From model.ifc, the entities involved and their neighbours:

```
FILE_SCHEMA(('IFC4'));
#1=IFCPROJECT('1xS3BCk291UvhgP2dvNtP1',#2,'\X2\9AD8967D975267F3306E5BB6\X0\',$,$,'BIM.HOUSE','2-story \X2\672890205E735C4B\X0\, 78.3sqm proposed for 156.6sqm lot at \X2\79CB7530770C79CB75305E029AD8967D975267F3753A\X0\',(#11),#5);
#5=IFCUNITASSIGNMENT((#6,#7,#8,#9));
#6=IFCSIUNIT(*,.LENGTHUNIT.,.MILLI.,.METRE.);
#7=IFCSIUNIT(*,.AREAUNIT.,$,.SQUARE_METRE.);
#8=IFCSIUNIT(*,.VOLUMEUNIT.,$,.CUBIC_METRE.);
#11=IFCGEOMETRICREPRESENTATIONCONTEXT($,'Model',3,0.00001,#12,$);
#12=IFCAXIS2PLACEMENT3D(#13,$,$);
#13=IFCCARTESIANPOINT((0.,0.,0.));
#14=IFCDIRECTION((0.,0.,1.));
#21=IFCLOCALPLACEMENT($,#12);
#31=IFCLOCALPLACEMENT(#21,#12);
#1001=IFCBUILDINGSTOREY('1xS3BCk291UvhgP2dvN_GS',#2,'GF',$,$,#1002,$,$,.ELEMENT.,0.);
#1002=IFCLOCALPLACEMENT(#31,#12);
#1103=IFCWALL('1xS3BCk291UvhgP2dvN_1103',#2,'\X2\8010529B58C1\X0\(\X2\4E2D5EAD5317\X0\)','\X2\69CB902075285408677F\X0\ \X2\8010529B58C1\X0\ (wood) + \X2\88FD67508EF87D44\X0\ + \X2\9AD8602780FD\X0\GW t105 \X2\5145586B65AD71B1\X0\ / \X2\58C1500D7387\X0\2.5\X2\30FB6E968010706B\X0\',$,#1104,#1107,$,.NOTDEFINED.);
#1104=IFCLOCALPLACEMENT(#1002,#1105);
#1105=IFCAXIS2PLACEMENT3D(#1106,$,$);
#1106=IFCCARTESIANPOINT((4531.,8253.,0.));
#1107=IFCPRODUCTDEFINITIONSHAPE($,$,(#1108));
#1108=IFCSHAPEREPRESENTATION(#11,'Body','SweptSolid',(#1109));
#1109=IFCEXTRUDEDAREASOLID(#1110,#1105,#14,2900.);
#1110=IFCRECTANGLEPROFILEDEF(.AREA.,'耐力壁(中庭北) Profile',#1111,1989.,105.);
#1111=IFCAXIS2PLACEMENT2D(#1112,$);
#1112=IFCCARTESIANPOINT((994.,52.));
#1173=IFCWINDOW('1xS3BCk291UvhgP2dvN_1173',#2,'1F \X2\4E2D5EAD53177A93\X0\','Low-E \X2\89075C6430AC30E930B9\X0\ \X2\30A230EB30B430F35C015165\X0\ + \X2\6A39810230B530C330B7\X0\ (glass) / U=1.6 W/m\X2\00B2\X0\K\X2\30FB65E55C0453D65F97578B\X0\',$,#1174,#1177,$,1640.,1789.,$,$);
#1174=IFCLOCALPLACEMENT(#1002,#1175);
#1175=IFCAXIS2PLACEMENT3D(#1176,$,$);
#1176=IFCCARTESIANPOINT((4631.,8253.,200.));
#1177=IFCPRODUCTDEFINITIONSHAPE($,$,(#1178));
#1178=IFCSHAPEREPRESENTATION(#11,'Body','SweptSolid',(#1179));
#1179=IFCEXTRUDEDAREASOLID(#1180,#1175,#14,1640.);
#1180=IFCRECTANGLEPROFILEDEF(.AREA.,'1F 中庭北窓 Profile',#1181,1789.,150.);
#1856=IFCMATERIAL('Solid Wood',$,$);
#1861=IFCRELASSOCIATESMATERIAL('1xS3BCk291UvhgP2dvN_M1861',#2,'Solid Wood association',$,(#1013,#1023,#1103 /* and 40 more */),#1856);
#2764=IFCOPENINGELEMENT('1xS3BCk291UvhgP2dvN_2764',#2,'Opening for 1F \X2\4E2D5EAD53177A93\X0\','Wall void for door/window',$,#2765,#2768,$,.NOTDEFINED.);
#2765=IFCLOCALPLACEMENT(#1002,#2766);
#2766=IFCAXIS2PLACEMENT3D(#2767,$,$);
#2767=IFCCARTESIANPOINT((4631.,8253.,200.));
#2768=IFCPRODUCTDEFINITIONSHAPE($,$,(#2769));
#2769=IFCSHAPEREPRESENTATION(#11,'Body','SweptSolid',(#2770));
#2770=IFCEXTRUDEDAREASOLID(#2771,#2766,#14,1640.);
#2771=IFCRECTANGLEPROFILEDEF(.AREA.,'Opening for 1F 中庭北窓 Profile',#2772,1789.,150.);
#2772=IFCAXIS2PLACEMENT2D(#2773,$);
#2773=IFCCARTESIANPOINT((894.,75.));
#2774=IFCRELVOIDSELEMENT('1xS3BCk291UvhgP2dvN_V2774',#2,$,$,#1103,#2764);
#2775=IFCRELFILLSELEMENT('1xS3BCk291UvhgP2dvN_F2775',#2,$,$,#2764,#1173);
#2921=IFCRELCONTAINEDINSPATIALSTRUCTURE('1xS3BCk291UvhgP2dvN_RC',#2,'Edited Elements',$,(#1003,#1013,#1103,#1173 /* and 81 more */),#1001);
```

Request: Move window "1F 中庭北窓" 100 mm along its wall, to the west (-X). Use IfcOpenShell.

```python
import ifcopenshell
import ifcopenshell.api.geometry
import ifcopenshell.util.placement

model = ifcopenshell.open("model.ifc")

window = model.by_guid("1xS3BCk291UvhgP2dvN_1173")
opening = window.FillsVoids[0].RelatingOpeningElement
wall = opening.VoidsElements[0].RelatingBuildingElement

wall_matrix = ifcopenshell.util.placement.get_local_placement(wall.ObjectPlacement)
shift = wall_matrix[:3, 0] * -100.0
before = ifcopenshell.util.placement.get_local_placement(window.ObjectPlacement)[:3, 3].copy()

# The window is not placed relative to its opening, so move both.
for product in (opening, window):
    matrix = ifcopenshell.util.placement.get_local_placement(product.ObjectPlacement)
    matrix[:3, 3] += shift
    ifcopenshell.api.geometry.edit_object_placement(model, product=product, matrix=matrix, is_si=False)

after = ifcopenshell.util.placement.get_local_placement(window.ObjectPlacement)[:3, 3]
print("window moved by", (after - before).round(3) + 0.0)

model.write("model_updated.ifc")
```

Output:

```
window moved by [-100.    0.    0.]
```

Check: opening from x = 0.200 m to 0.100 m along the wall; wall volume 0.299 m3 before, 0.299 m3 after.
